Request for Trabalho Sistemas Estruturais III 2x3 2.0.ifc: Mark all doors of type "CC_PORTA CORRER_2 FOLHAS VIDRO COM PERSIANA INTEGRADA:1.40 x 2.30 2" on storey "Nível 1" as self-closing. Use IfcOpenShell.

First a look at what the model holds.

```python
import ifcopenshell
import ifcopenshell.util.element

model = ifcopenshell.open("Trabalho Sistemas Estruturais III 2x3 2.0.ifc")
print(model.schema)
storey = next(s for s in model.by_type("IfcBuildingStorey") if s.Name == "Nível 1")
doors = [e for e in ifcopenshell.util.element.get_decomposition(storey) if e.is_a("IfcDoor")]
seen = {}
for e in doors:
    element_type = ifcopenshell.util.element.get_type(e)
    key = (element_type.Name if element_type != e and element_type else None, ifcopenshell.util.element.get_pset(e, "Pset_DoorCommon", "SelfClosing"))
    seen[key] = seen.get(key, 0) + 1
for (name, value), count in sorted(seen.items(), key=str):
    print(count, "x", name, "|", value)
```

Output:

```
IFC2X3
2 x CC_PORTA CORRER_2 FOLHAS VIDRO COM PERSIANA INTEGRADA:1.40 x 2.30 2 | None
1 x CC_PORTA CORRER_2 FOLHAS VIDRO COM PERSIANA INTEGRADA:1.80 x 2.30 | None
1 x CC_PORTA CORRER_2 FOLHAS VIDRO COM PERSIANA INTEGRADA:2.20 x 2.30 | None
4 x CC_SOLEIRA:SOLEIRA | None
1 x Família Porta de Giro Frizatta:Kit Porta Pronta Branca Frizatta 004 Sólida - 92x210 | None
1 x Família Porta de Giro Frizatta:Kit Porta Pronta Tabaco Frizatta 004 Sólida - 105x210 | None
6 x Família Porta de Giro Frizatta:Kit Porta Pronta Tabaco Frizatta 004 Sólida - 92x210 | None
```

```python
import ifcopenshell
import ifcopenshell.api.pset
import ifcopenshell.util.element

model = ifcopenshell.open("Trabalho Sistemas Estruturais III 2x3 2.0.ifc")

storey = next(s for s in model.by_type("IfcBuildingStorey") if s.Name == "Nível 1")
doors = [e for e in ifcopenshell.util.element.get_decomposition(storey) if e.is_a("IfcDoor")]

count = 0
for e in doors:
    element_type = ifcopenshell.util.element.get_type(e)
    if element_type in (None, e) or element_type.Name != "CC_PORTA CORRER_2 FOLHAS VIDRO COM PERSIANA INTEGRADA:1.40 x 2.30 2":
        continue
    # add_pset returns the element's existing set when there is one.
    pset = ifcopenshell.api.pset.add_pset(model, product=e, name="Pset_DoorCommon")
    ifcopenshell.api.pset.edit_pset(model, pset=pset, properties={"SelfClosing": True})
    count += 1

print(count, "doors updated")

model.write("Trabalho Sistemas Estruturais III 2x3 2.0_rev.ifc")
```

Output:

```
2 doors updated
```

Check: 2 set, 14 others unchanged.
